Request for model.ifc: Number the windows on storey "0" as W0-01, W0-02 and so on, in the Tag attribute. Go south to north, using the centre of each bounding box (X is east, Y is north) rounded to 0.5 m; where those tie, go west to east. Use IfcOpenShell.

First a look at what the model holds.

```python
import ifcopenshell
import ifcopenshell.util.element
import ifcopenshell.util.placement

model = ifcopenshell.open("model.ifc")
print(model.schema)
storey = next(s for s in model.by_type("IfcBuildingStorey") if s.Name == "0")
windows = [e for e in ifcopenshell.util.element.get_decomposition(storey) if e.is_a("IfcWindow")]
for e in sorted(windows, key=lambda e: e.id()):
    origin = ifcopenshell.util.placement.get_local_placement(e.ObjectPlacement)[:3, 3]
    print(e.id(), e.Tag, e.Name, origin.round(2) + 0.0, sep=" | ")
```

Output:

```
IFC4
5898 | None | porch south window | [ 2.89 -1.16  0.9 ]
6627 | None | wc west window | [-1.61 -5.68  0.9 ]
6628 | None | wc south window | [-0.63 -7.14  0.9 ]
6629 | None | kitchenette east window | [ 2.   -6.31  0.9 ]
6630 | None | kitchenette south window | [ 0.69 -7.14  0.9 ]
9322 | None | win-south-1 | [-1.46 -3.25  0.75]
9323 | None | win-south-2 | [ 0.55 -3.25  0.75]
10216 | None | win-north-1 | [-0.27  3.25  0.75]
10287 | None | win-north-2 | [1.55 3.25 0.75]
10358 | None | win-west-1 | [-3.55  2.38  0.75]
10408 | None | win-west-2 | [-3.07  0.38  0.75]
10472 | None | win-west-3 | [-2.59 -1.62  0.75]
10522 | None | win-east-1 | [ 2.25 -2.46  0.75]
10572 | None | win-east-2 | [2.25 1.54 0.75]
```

```python
import ifcopenshell
import ifcopenshell.geom
import ifcopenshell.util.element
import ifcopenshell.util.shape

model = ifcopenshell.open("model.ifc")
settings = ifcopenshell.geom.settings()
settings.set("use-world-coords", True)


def centre(element):
    shape = ifcopenshell.geom.create_shape(settings, element)
    return ifcopenshell.util.shape.get_bbox_centroid(shape.geometry)


storey = next(s for s in model.by_type("IfcBuildingStorey") if s.Name == "0")
windows = [e for e in ifcopenshell.util.element.get_decomposition(storey) if e.is_a("IfcWindow")]

# Insertion points can sit at a corner or the storey origin, so sort by the geometry (in metres).
centres = {e: centre(e) for e in windows}
windows.sort(key=lambda e: (round(centres[e][1] / 0.5), centres[e][0]))

for i, e in enumerate(windows, start=1):
    number = f"W0-{i:02d}"
    e.Tag = number
    print(e.id(), number)

model.write("model_v2.ifc")
```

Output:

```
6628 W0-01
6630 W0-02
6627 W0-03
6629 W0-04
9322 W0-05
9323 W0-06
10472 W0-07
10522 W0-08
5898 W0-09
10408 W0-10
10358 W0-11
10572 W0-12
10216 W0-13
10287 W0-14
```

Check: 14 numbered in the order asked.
